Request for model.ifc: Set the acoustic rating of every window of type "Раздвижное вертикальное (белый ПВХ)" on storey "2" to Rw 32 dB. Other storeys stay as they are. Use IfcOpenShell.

First a look at what the model holds.

```python
import ifcopenshell
import ifcopenshell.util.element

model = ifcopenshell.open("model.ifc")
print(model.schema)
storey = next(s for s in model.by_type("IfcBuildingStorey") if s.Name == "2")
windows = [e for e in ifcopenshell.util.element.get_decomposition(storey) if e.is_a("IfcWindow")]
seen = {}
for e in windows:
    element_type = ifcopenshell.util.element.get_type(e)
    key = (element_type.Name if element_type != e and element_type else None, ifcopenshell.util.element.get_pset(e, "Pset_WindowCommon", "AcousticRating"))
    seen[key] = seen.get(key, 0) + 1
for (name, value), count in sorted(seen.items(), key=str):
    print(count, "x", name, "|", value)
```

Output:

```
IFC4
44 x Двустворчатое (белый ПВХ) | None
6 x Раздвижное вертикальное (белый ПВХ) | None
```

```python
import ifcopenshell
import ifcopenshell.api.pset
import ifcopenshell.util.element

model = ifcopenshell.open("model.ifc")

storey = next(s for s in model.by_type("IfcBuildingStorey") if s.Name == "2")
windows = [e for e in ifcopenshell.util.element.get_decomposition(storey) if e.is_a("IfcWindow")]

count = 0
for e in windows:
    element_type = ifcopenshell.util.element.get_type(e)
    if element_type in (None, e) or element_type.Name != "Раздвижное вертикальное (белый ПВХ)":
        continue
    # add_pset returns the element's existing set when there is one.
    pset = ifcopenshell.api.pset.add_pset(model, product=e, name="Pset_WindowCommon")
    ifcopenshell.api.pset.edit_pset(model, pset=pset, properties={"AcousticRating": "Rw 32 dB"})
    count += 1

print(count, "windows updated")

model.write("model-out.ifc")
```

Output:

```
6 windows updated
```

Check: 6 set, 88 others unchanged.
